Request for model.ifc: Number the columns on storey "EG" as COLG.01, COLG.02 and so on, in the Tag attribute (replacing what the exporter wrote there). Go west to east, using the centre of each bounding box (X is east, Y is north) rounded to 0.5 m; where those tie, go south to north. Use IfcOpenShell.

First a look at what the model holds.

```python
import ifcopenshell
import ifcopenshell.util.element
import ifcopenshell.util.placement

model = ifcopenshell.open("model.ifc")
print(model.schema)
storey = next(s for s in model.by_type("IfcBuildingStorey") if s.Name == "EG")
columns = [e for e in ifcopenshell.util.element.get_decomposition(storey) if e.is_a("IfcColumn")]
for e in sorted(columns, key=lambda e: e.id()):
    origin = ifcopenshell.util.placement.get_local_placement(e.ObjectPlacement)[:3, 3]
    print(e.id(), e.Tag, e.Name, origin.round(2) + 0.0, sep=" | ")
```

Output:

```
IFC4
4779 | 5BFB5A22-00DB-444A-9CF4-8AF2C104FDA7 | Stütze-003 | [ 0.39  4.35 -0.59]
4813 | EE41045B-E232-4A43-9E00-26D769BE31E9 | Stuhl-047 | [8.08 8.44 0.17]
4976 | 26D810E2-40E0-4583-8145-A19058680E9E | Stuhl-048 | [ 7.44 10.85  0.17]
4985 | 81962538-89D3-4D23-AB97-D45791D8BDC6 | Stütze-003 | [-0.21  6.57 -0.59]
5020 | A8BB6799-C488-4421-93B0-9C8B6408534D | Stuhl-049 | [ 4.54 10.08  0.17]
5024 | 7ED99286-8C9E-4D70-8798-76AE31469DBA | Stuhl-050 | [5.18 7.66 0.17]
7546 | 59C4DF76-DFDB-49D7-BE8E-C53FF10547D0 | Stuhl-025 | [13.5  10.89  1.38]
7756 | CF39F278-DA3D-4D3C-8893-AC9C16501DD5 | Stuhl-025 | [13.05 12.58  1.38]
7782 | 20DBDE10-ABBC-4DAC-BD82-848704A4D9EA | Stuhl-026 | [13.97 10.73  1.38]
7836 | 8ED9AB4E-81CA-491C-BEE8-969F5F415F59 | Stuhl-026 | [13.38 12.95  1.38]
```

```python
import ifcopenshell
import ifcopenshell.geom
import ifcopenshell.util.element
import ifcopenshell.util.shape

model = ifcopenshell.open("model.ifc")
settings = ifcopenshell.geom.settings()
settings.set("use-world-coords", True)


def centre(element):
    shape = ifcopenshell.geom.create_shape(settings, element)
    return ifcopenshell.util.shape.get_bbox_centroid(shape.geometry)


storey = next(s for s in model.by_type("IfcBuildingStorey") if s.Name == "EG")
columns = [e for e in ifcopenshell.util.element.get_decomposition(storey) if e.is_a("IfcColumn")]

# Insertion points can sit at a corner or the storey origin, so sort by the geometry (in metres).
centres = {e: centre(e) for e in columns}
columns.sort(key=lambda e: (round(centres[e][0] / 0.5), centres[e][1]))

for i, e in enumerate(columns, start=1):
    number = f"COLG.{i:02d}"
    e.Tag = number
    print(e.id(), number)

model.write("model-out.ifc")
```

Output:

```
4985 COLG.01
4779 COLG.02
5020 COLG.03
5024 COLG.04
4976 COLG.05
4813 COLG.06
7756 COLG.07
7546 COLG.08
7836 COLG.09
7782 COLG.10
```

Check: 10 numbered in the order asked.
